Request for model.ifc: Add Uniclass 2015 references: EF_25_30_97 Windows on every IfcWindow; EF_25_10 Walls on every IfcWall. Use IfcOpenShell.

First a look at what the model holds.

```python
import ifcopenshell

model = ifcopenshell.open("model.ifc")
print(model.schema)
print("classifications:", [c.Name for c in model.by_type("IfcClassification")])
for ifc_class in ("IfcDoor", "IfcRoof", "IfcStair", "IfcWall", "IfcWindow"):
    print(ifc_class, len(model.by_type(ifc_class)))
```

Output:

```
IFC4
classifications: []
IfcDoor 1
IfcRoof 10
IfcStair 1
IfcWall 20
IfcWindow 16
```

```python
import ifcopenshell
import ifcopenshell.api.classification

model = ifcopenshell.open("model.ifc")

system = ifcopenshell.api.classification.add_classification(model, classification="Uniclass 2015")

codes = {
    "IfcWindow": ("EF_25_30_97", "Windows"),
    "IfcWall": ("EF_25_10", "Walls"),
}
for ifc_class, (code, name) in codes.items():
    products = model.by_type(ifc_class)
    ifcopenshell.api.classification.add_reference(
        model, products=products, classification=system, identification=code, name=name
    )
    print(code, len(products))

model.write("model_rev.ifc")
```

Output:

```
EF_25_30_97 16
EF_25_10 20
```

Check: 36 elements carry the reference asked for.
